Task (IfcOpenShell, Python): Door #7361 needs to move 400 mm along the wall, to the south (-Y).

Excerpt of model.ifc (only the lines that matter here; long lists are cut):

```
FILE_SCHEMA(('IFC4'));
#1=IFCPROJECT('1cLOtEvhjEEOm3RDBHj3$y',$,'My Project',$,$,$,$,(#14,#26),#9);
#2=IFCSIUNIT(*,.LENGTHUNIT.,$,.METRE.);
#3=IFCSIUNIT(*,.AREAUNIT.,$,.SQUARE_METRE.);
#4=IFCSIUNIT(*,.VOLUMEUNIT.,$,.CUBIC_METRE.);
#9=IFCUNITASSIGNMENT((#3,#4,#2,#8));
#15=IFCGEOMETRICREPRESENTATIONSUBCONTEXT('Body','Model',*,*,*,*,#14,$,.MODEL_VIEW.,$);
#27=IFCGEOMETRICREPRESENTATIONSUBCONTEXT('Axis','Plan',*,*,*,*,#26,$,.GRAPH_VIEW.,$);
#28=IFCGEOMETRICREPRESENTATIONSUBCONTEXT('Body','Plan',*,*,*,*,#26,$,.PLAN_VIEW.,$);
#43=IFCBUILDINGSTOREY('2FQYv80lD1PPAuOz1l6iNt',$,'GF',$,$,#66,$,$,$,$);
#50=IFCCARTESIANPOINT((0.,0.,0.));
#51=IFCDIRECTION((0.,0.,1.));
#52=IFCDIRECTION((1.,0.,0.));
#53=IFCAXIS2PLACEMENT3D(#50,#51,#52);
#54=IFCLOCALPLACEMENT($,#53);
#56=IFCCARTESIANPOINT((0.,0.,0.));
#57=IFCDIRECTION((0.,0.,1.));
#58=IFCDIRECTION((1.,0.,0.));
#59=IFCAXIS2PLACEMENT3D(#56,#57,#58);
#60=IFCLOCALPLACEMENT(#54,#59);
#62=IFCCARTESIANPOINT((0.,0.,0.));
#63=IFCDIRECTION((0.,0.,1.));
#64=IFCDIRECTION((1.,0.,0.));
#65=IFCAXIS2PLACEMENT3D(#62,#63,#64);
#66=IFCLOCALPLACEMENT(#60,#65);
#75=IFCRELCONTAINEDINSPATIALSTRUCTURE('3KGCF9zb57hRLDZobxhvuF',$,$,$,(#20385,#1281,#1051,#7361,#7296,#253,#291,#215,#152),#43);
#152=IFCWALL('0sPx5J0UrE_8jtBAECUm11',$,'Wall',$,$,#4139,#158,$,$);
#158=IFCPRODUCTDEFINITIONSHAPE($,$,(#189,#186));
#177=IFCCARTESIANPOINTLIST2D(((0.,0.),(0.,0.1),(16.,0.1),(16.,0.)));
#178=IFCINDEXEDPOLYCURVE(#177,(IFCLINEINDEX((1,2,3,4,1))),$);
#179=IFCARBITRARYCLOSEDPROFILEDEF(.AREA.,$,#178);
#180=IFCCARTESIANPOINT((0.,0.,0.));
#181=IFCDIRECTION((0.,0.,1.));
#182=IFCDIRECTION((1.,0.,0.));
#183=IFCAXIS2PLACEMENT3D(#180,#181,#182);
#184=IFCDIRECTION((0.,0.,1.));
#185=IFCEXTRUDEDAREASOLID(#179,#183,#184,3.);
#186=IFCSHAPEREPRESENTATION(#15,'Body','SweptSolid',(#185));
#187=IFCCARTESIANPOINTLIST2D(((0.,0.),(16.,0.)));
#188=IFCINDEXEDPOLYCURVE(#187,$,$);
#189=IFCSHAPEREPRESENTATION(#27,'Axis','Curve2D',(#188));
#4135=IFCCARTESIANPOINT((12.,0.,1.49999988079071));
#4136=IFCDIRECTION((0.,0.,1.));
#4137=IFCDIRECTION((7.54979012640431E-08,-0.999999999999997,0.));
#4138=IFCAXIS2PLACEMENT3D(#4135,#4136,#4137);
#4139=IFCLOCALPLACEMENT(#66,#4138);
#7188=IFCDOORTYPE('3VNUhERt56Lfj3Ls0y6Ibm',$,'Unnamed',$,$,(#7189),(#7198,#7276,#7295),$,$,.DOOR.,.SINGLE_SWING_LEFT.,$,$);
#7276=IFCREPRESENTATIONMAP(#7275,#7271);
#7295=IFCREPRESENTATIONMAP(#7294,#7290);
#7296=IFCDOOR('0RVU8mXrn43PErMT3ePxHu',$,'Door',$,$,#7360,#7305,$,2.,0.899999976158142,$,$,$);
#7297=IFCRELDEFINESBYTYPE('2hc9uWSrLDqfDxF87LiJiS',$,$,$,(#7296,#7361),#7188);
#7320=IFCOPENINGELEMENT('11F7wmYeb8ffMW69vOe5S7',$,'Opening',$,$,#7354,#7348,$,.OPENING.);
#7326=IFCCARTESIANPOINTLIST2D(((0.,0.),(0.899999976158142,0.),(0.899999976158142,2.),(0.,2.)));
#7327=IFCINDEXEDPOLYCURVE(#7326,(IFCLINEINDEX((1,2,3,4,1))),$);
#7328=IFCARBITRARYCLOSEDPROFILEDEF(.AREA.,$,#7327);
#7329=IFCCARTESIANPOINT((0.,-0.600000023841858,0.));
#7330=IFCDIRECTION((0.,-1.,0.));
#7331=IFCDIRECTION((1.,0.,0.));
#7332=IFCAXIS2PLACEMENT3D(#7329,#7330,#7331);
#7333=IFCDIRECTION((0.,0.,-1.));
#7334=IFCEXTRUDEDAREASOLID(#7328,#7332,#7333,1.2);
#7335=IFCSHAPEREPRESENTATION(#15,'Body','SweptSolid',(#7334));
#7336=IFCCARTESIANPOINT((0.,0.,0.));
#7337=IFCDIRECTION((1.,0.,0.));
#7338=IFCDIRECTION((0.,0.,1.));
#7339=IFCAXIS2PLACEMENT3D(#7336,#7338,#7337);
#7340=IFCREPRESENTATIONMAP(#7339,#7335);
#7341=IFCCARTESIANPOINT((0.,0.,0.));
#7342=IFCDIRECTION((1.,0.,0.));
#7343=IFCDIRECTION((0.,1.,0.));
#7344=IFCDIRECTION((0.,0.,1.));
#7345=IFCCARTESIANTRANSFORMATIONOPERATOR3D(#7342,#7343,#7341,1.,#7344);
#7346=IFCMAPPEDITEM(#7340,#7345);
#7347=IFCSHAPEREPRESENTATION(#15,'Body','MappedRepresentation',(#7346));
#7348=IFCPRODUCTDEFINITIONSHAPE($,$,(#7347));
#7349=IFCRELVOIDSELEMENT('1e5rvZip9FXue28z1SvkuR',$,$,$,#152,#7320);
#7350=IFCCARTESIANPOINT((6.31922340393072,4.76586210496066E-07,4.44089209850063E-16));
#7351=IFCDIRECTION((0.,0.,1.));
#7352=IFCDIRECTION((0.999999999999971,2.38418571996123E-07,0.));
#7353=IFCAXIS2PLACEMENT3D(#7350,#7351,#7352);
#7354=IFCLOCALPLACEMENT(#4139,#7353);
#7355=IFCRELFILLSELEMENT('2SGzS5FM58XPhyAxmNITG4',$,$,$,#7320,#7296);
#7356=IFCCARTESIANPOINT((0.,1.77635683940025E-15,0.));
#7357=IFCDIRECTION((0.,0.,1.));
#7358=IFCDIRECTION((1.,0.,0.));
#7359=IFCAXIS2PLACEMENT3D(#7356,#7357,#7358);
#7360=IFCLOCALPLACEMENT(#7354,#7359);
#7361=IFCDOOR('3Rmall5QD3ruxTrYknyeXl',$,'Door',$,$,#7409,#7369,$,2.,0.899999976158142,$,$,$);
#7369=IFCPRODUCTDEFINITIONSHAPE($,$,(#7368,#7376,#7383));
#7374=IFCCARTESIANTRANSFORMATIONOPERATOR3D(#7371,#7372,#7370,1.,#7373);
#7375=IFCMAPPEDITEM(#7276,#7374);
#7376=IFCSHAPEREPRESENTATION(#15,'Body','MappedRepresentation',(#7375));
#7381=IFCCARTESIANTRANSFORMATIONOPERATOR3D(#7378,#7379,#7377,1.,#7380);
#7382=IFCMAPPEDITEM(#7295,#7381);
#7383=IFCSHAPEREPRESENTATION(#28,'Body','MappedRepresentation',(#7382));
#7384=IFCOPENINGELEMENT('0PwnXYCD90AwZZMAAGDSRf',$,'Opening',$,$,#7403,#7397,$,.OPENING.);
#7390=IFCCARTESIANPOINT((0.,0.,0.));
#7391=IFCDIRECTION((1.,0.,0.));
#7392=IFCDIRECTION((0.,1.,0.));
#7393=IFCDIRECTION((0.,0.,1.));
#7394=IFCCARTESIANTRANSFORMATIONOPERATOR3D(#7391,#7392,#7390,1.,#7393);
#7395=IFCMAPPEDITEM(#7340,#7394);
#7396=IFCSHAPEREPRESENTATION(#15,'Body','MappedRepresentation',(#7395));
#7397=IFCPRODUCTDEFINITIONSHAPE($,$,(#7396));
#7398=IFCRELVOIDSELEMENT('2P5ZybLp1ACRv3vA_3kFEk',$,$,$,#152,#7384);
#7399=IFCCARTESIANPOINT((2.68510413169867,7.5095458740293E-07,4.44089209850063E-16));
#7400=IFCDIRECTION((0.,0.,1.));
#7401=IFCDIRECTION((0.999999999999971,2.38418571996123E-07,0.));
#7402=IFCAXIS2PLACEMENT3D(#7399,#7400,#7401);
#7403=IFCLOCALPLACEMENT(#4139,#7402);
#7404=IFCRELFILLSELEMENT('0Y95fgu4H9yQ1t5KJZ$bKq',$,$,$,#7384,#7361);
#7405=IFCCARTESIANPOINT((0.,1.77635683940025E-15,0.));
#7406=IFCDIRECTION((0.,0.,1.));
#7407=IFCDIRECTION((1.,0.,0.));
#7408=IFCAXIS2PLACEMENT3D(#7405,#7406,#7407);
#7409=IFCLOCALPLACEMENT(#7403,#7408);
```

```python
import ifcopenshell
import ifcopenshell.api.geometry
import ifcopenshell.util.placement
import ifcopenshell.util.unit

model = ifcopenshell.open("model.ifc")
unit_scale = ifcopenshell.util.unit.calculate_unit_scale(model)

door = model.by_guid("3Rmall5QD3ruxTrYknyeXl")
opening = door.FillsVoids[0].RelatingOpeningElement
wall = opening.VoidsElements[0].RelatingBuildingElement

wall_matrix = ifcopenshell.util.placement.get_local_placement(wall.ObjectPlacement)
shift = wall_matrix[:3, 0] * 0.4 / unit_scale
before = ifcopenshell.util.placement.get_local_placement(door.ObjectPlacement)[:3, 3].copy()

# The door is placed relative to its opening, so it follows when the opening moves.
matrix = ifcopenshell.util.placement.get_local_placement(opening.ObjectPlacement)
matrix[:3, 3] += shift
ifcopenshell.api.geometry.edit_object_placement(
    model, product=opening, matrix=matrix, is_si=False, should_transform_children=True
)

after = ifcopenshell.util.placement.get_local_placement(door.ObjectPlacement)[:3, 3]
print("door moved by", (after - before).round(3) + 0.0)

model.write("model_edited.ifc")
```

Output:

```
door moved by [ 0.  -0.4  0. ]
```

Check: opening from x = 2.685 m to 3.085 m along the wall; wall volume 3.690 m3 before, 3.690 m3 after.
